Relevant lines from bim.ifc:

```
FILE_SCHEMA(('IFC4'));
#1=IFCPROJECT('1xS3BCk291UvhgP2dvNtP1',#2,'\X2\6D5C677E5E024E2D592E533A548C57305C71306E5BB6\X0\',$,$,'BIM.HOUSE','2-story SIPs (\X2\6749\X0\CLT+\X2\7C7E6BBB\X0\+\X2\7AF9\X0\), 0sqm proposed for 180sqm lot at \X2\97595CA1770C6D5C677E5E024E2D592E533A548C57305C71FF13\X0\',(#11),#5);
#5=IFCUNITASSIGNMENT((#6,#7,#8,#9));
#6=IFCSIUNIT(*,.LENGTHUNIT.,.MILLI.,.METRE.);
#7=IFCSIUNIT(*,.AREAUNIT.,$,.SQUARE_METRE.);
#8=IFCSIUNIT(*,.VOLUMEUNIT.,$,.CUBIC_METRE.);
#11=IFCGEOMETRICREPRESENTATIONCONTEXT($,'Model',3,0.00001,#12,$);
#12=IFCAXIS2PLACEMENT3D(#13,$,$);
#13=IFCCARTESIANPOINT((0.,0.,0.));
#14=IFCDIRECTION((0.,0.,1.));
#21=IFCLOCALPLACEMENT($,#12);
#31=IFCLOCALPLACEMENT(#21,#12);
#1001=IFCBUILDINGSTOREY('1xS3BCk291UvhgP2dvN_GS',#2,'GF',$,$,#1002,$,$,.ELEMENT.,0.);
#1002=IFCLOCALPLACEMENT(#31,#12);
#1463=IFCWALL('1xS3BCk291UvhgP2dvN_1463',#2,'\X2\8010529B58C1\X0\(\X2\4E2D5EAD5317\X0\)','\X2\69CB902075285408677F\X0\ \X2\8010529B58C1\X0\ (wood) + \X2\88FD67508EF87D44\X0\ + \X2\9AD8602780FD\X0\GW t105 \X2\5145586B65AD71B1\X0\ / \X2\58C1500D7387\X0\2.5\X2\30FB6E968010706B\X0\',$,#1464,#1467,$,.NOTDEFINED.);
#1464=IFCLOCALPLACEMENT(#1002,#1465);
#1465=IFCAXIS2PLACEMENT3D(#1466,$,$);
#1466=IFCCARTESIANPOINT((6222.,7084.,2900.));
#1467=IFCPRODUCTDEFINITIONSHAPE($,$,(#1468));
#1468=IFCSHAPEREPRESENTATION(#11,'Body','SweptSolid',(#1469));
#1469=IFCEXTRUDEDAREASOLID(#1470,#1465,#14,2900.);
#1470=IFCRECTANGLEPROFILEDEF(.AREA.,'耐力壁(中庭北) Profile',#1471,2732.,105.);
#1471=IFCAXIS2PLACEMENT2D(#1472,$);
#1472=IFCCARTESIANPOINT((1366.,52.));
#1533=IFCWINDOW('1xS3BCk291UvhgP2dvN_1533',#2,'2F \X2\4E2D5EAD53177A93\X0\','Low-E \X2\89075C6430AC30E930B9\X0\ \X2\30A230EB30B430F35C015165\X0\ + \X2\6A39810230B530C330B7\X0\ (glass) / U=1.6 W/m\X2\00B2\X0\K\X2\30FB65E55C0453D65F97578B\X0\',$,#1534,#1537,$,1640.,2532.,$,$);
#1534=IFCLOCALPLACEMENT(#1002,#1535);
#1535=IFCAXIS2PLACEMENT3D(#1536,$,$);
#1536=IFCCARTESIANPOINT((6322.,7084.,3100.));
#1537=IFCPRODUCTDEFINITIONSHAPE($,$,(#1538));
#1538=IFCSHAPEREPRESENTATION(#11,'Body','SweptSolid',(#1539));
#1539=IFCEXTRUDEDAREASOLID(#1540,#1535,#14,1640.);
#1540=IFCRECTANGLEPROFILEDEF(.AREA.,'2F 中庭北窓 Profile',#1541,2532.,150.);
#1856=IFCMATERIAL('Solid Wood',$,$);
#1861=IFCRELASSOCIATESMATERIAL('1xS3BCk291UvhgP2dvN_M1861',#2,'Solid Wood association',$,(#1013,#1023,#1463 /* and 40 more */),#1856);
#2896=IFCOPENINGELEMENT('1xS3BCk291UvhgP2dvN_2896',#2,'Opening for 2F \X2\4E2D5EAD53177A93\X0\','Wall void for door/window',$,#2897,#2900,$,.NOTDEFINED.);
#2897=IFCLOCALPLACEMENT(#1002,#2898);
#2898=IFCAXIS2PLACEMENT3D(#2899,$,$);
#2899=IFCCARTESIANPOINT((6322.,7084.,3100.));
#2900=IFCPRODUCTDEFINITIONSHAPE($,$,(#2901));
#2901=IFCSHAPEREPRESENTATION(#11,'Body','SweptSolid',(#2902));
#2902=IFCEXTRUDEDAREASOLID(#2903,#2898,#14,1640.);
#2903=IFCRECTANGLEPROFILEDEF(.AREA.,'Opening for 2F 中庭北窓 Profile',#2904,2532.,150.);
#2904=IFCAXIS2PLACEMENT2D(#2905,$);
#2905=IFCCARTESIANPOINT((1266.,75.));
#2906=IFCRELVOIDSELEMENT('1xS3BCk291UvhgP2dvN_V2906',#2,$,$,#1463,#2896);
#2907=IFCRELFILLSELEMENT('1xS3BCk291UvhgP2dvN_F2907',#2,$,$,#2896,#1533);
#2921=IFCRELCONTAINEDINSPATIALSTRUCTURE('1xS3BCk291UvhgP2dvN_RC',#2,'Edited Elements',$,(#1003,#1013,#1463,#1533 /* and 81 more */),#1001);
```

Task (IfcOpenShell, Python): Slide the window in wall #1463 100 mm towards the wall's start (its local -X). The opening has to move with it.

```python
import ifcopenshell
import ifcopenshell.api.geometry
import ifcopenshell.util.placement
import ifcopenshell.util.unit

model = ifcopenshell.open("bim.ifc")
unit_scale = ifcopenshell.util.unit.calculate_unit_scale(model)

window = model.by_id(1533)
opening = window.FillsVoids[0].RelatingOpeningElement
wall = opening.VoidsElements[0].RelatingBuildingElement

wall_matrix = ifcopenshell.util.placement.get_local_placement(wall.ObjectPlacement)
shift = wall_matrix[:3, 0] * -0.1 / unit_scale
before = ifcopenshell.util.placement.get_local_placement(window.ObjectPlacement)[:3, 3].copy()

# The window is not placed relative to its opening, so move both.
for product in (opening, window):
    matrix = ifcopenshell.util.placement.get_local_placement(product.ObjectPlacement)
    matrix[:3, 3] += shift
    ifcopenshell.api.geometry.edit_object_placement(model, product=product, matrix=matrix, is_si=False)

after = ifcopenshell.util.placement.get_local_placement(window.ObjectPlacement)[:3, 3]
print("window moved by", (after - before).round(3) + 0.0)

model.write("bim_rev.ifc")
```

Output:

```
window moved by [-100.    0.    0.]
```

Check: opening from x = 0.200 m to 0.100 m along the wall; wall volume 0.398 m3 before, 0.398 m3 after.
